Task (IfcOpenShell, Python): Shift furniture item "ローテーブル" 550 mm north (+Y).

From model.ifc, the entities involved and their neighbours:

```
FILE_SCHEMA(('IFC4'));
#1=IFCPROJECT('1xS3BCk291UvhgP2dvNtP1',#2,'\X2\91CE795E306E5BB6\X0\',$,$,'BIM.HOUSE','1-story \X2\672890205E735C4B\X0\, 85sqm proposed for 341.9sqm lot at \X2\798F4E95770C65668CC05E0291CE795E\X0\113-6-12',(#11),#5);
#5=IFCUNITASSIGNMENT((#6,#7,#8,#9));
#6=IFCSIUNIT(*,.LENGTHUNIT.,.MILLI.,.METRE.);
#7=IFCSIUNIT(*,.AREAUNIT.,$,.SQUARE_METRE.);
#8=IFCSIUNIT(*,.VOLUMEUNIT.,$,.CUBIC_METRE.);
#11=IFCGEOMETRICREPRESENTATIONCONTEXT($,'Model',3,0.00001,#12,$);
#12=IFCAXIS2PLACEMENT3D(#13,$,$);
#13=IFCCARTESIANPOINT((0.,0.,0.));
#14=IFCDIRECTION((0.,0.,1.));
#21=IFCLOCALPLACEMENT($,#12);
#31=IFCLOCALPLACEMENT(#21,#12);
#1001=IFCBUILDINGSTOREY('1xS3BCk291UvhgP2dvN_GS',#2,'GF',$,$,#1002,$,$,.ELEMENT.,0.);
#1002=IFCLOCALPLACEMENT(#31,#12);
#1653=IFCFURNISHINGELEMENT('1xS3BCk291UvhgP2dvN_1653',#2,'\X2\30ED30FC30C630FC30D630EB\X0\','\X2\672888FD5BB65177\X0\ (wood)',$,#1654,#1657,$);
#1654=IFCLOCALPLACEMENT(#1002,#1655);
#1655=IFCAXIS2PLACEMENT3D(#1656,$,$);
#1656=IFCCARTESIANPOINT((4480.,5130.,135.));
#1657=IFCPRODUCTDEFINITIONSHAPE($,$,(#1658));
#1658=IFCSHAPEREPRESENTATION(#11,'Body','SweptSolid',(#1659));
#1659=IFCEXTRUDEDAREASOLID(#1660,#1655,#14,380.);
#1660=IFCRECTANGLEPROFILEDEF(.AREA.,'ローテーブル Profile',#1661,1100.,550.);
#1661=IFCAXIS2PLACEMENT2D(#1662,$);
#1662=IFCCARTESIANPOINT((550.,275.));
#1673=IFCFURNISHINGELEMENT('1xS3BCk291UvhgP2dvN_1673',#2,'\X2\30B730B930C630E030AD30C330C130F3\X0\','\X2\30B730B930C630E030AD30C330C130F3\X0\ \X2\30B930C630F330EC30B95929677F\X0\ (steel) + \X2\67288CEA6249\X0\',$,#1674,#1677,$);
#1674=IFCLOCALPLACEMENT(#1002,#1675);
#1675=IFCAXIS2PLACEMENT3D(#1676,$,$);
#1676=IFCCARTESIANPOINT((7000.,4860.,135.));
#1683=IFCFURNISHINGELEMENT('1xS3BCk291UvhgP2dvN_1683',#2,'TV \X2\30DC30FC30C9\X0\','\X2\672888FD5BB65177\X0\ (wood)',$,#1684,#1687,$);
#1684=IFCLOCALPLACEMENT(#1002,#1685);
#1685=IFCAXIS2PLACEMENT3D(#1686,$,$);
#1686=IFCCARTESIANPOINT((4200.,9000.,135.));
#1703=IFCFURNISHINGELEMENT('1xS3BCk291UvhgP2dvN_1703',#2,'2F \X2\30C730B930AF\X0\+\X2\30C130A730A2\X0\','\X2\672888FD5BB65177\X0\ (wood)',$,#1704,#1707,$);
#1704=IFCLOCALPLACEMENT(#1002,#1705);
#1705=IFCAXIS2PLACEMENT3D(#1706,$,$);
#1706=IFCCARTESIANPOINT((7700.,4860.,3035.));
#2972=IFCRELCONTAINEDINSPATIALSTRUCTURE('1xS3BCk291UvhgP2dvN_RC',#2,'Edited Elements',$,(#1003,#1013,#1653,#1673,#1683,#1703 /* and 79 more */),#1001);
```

```python
import ifcopenshell
import ifcopenshell.api.geometry
import ifcopenshell.util.placement
import ifcopenshell.util.unit

model = ifcopenshell.open("model.ifc")
unit_scale = ifcopenshell.util.unit.calculate_unit_scale(model)

item = model.by_guid("1xS3BCk291UvhgP2dvN_1653")
matrix = ifcopenshell.util.placement.get_local_placement(item.ObjectPlacement)
matrix[1, 3] += 0.55 / unit_scale
ifcopenshell.api.geometry.edit_object_placement(model, product=item, matrix=matrix, is_si=False)

print(ifcopenshell.util.placement.get_local_placement(item.ObjectPlacement).round(3) + 0.0)

model.write("model_updated.ifc")
```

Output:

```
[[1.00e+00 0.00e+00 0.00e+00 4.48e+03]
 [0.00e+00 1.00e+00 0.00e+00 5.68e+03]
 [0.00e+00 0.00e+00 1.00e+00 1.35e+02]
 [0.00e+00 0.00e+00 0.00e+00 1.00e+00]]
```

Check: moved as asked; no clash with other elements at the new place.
